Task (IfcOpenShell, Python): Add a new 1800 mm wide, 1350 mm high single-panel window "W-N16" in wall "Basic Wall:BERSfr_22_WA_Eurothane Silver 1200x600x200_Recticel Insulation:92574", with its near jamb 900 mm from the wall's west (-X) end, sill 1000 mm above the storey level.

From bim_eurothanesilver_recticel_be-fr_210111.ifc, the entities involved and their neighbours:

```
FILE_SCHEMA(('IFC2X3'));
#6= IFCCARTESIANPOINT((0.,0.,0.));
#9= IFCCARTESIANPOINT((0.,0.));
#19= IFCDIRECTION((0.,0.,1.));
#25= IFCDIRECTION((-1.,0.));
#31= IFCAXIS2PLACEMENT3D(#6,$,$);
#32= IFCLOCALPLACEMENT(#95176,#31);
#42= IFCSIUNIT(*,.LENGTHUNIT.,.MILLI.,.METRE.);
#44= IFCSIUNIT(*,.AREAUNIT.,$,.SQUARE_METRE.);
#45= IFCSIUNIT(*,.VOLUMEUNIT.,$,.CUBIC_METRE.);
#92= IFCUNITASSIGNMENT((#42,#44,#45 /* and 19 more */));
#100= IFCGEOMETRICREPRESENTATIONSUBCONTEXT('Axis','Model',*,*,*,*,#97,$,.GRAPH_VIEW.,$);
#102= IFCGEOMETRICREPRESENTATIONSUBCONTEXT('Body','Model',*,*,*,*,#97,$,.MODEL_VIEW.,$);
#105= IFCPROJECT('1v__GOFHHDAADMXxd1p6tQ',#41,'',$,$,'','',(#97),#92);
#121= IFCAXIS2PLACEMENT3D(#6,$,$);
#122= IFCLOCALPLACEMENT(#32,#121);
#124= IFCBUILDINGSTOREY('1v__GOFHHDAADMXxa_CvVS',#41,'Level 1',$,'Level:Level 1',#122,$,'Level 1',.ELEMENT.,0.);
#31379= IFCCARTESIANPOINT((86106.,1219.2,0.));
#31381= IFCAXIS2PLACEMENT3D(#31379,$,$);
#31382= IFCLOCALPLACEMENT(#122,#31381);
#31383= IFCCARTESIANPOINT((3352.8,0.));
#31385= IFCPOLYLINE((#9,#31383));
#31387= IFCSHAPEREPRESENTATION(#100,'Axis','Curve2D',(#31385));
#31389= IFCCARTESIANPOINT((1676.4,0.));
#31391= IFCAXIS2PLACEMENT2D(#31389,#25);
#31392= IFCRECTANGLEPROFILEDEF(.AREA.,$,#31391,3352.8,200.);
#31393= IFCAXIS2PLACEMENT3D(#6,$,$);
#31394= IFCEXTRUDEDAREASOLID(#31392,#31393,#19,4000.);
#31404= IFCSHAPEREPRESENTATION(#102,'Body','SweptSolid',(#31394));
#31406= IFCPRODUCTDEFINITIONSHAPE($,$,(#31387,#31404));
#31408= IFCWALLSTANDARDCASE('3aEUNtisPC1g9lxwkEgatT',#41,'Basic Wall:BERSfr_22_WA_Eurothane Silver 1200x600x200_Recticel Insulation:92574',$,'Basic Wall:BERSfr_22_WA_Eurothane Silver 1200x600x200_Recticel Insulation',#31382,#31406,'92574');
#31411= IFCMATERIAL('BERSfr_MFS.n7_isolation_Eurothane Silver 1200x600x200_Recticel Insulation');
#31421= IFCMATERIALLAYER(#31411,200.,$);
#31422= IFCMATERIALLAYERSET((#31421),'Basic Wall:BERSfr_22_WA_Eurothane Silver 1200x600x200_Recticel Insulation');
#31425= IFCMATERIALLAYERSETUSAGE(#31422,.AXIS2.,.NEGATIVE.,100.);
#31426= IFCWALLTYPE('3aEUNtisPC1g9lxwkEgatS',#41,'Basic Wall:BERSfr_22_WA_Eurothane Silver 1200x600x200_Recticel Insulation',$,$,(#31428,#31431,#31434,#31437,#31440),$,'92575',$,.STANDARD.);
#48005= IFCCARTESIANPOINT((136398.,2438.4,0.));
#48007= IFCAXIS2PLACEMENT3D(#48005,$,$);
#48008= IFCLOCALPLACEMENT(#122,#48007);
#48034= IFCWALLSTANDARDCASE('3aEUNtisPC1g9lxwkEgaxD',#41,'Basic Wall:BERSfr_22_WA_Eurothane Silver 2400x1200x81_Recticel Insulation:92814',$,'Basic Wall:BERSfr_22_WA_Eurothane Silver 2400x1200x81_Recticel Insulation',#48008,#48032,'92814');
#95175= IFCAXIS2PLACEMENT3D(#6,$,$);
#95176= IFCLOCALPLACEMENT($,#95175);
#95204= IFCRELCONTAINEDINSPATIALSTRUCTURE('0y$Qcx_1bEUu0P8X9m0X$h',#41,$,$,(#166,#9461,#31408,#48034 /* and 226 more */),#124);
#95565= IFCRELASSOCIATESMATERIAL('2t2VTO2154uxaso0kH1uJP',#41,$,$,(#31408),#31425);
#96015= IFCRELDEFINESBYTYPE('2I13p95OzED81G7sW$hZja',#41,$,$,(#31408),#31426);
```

```python
import numpy as np
import ifcopenshell
import ifcopenshell.api.feature
import ifcopenshell.api.geometry
import ifcopenshell.api.root
import ifcopenshell.api.spatial
import ifcopenshell.api.type
import ifcopenshell.geom
import ifcopenshell.util.element
import ifcopenshell.util.placement
import ifcopenshell.util.representation
import ifcopenshell.util.shape
import ifcopenshell.util.unit

model = ifcopenshell.open("bim_eurothanesilver_recticel_be-fr_210111.ifc")
unit_scale = ifcopenshell.util.unit.calculate_unit_scale(model)
settings = ifcopenshell.geom.settings()


def volume(element):
    """Net volume in cubic metres, openings subtracted."""
    shape = ifcopenshell.geom.create_shape(settings, element)
    return ifcopenshell.util.shape.get_volume(shape.geometry)


wall = model.by_guid("3aEUNtisPC1g9lxwkEgatT")
storey = ifcopenshell.util.element.get_container(wall, ifc_class="IfcBuildingStorey")
context = ifcopenshell.util.representation.get_context(model, "Model", "Body", "MODEL_VIEW")
before = volume(wall)

width, height, from_end, sill = 1.8, 1.35, 0.9, 1  # metres

# The wall runs along its own X axis, and the end named is its -X end.
wall_shape = ifcopenshell.geom.create_shape(settings, wall)
x, y, z = ifcopenshell.util.shape.get_vertices(wall_shape.geometry).T
start = x.min() + from_end
face, thickness = float(y.min()), float(y.max() - y.min())
wall_matrix = ifcopenshell.util.placement.get_local_placement(wall.ObjectPlacement)
level = ifcopenshell.util.placement.get_local_placement(storey.ObjectPlacement)[2, 3]


def in_wall(x, y):
    """Placement at x, y metres in the wall's axes, at sill height."""
    matrix = wall_matrix.copy()
    matrix[:, 3] = wall_matrix @ np.array([x / unit_scale, y / unit_scale, 0.0, 1.0])
    matrix[2, 3] = level + sill / unit_scale
    return matrix


# Opening: a box that overshoots both wall faces by 50 mm.
opening = ifcopenshell.api.root.create_entity(model, ifc_class="IfcOpeningElement")
box = ifcopenshell.api.geometry.add_wall_representation(
    model, context=context, length=width, height=height, thickness=thickness + 0.1
)
ifcopenshell.api.geometry.assign_representation(model, product=opening, representation=box)
ifcopenshell.api.geometry.edit_object_placement(model, product=opening, matrix=in_wall(start, face - 0.05), is_si=False)
ifcopenshell.api.feature.add_feature(model, feature=opening, element=wall)

window = ifcopenshell.api.root.create_entity(model, ifc_class="IfcWindow", name="W-N16")
window.OverallWidth, window.OverallHeight = width / unit_scale, height / unit_scale
body = ifcopenshell.api.geometry.add_window_representation(
    model,
    context=context,
    overall_width=window.OverallWidth,
    overall_height=window.OverallHeight,
    partition_type="SINGLE_PANEL",
)
ifcopenshell.api.geometry.assign_representation(model, product=window, representation=body)
ifcopenshell.api.spatial.assign_container(model, products=[window], relating_structure=storey)
fills = ifcopenshell.api.feature.add_filling(model, opening=opening, element=window)
fills.OwnerHistory = window.OwnerHistory  # required in IFC2X3

# IFC2X3 keeps the operation on the window style.
style = ifcopenshell.api.root.create_entity(model, ifc_class="IfcWindowStyle", name="W-N16")
style.OperationType, style.ConstructionType = "SINGLE_PANEL", "NOTDEFINED"
style.ParameterTakesPrecedence = style.Sizeable = False
ifcopenshell.api.type.assign_type(model, related_objects=[window], relating_type=style)

# Centre the window in the wall's thickness.
ifcopenshell.api.geometry.edit_object_placement(model, product=window, matrix=in_wall(start, face), is_si=False)
window_shape = ifcopenshell.geom.create_shape(settings, window)
depth = ifcopenshell.util.shape.get_vertices(window_shape.geometry)[:, 1]
offset = face + thickness / 2 - (depth.min() + depth.max()) / 2
ifcopenshell.api.geometry.edit_object_placement(model, product=window, matrix=in_wall(start, offset), is_si=False)

after = volume(wall)

print(f"wall volume {before:.3f} -> {after:.3f} m3")

model.write("bim_eurothanesilver_recticel_be-fr_210111_v2.ifc")
```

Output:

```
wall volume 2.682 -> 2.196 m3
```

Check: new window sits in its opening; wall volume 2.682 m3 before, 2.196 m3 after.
